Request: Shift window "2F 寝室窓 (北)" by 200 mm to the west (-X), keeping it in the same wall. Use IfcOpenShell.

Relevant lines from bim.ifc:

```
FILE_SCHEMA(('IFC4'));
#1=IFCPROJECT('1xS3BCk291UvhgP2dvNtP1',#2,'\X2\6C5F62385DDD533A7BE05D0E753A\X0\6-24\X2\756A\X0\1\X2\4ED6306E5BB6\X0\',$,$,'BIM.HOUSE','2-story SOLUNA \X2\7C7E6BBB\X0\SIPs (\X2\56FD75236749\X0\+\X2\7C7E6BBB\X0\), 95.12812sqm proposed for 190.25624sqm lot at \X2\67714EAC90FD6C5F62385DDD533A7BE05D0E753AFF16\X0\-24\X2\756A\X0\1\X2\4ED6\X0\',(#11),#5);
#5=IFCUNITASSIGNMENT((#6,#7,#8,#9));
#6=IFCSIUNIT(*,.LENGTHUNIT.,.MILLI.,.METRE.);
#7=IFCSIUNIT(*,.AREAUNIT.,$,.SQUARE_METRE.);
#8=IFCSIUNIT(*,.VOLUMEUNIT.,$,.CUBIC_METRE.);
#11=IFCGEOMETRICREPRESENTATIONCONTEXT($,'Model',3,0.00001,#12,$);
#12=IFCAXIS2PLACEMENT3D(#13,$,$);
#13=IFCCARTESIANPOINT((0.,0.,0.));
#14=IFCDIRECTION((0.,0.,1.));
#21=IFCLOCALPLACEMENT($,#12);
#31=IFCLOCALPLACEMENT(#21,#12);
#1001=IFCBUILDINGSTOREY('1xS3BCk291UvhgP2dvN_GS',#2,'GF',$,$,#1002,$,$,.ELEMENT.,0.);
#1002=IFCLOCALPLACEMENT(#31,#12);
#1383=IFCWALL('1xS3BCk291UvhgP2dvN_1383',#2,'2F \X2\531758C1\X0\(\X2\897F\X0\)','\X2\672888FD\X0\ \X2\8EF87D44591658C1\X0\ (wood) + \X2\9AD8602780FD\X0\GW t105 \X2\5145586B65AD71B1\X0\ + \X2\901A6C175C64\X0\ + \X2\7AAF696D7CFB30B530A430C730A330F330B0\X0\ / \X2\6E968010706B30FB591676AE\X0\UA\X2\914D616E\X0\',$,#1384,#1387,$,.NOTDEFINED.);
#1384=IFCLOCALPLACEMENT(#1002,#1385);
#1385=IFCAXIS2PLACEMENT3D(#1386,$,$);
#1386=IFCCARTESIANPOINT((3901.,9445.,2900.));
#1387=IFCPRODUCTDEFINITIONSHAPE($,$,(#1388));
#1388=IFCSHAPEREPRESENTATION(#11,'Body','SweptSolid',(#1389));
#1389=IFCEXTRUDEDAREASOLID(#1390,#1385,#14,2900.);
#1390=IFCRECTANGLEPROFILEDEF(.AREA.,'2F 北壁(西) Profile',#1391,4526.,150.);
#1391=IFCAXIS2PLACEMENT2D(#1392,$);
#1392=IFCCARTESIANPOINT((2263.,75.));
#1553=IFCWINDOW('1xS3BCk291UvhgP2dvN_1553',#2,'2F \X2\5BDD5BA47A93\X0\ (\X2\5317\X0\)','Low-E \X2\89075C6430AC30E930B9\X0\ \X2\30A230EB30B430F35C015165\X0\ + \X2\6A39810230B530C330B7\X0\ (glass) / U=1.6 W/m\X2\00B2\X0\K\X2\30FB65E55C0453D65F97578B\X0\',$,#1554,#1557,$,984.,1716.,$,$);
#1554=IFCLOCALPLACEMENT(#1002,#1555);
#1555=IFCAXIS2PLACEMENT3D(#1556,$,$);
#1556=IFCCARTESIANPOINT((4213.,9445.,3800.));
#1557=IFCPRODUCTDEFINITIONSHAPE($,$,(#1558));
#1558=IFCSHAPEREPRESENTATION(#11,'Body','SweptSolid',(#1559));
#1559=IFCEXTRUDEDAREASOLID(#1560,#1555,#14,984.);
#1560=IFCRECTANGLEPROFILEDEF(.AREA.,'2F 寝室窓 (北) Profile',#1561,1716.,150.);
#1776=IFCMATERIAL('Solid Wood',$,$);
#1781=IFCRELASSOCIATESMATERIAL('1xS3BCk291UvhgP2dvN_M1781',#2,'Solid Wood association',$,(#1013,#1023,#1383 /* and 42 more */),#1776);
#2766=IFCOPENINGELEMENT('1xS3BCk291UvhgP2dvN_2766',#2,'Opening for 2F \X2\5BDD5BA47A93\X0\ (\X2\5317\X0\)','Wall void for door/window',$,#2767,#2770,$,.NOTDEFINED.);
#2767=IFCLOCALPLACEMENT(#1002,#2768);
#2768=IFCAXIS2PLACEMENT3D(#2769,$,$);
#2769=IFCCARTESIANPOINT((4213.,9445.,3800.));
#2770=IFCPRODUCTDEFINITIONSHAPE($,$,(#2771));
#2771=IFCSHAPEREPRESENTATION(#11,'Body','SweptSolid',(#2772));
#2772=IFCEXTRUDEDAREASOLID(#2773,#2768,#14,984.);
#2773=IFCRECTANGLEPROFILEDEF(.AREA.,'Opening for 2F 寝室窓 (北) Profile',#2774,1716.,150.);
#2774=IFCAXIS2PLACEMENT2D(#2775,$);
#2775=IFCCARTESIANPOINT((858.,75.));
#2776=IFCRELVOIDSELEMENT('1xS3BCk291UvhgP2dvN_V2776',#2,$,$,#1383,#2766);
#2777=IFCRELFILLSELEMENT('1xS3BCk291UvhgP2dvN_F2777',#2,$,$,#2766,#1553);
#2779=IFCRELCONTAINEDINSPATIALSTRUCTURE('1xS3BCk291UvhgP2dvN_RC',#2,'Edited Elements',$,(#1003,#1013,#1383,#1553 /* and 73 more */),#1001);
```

```python
import ifcopenshell
import ifcopenshell.api.geometry
import ifcopenshell.util.placement
import ifcopenshell.util.unit

model = ifcopenshell.open("bim.ifc")
unit_scale = ifcopenshell.util.unit.calculate_unit_scale(model)

window = model.by_guid("1xS3BCk291UvhgP2dvN_1553")
opening = window.FillsVoids[0].RelatingOpeningElement
wall = opening.VoidsElements[0].RelatingBuildingElement

wall_matrix = ifcopenshell.util.placement.get_local_placement(wall.ObjectPlacement)
shift = wall_matrix[:3, 0] * -0.2 / unit_scale
before = ifcopenshell.util.placement.get_local_placement(window.ObjectPlacement)[:3, 3].copy()

# The window is not placed relative to its opening, so move both.
for product in (opening, window):
    matrix = ifcopenshell.util.placement.get_local_placement(product.ObjectPlacement)
    matrix[:3, 3] += shift
    ifcopenshell.api.geometry.edit_object_placement(model, product=product, matrix=matrix, is_si=False)

after = ifcopenshell.util.placement.get_local_placement(window.ObjectPlacement)[:3, 3]
print("window moved by", (after - before).round(3) + 0.0)

model.write("bim_updated.ifc")
```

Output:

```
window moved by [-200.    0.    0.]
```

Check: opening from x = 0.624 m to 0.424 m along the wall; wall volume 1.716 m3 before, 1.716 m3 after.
